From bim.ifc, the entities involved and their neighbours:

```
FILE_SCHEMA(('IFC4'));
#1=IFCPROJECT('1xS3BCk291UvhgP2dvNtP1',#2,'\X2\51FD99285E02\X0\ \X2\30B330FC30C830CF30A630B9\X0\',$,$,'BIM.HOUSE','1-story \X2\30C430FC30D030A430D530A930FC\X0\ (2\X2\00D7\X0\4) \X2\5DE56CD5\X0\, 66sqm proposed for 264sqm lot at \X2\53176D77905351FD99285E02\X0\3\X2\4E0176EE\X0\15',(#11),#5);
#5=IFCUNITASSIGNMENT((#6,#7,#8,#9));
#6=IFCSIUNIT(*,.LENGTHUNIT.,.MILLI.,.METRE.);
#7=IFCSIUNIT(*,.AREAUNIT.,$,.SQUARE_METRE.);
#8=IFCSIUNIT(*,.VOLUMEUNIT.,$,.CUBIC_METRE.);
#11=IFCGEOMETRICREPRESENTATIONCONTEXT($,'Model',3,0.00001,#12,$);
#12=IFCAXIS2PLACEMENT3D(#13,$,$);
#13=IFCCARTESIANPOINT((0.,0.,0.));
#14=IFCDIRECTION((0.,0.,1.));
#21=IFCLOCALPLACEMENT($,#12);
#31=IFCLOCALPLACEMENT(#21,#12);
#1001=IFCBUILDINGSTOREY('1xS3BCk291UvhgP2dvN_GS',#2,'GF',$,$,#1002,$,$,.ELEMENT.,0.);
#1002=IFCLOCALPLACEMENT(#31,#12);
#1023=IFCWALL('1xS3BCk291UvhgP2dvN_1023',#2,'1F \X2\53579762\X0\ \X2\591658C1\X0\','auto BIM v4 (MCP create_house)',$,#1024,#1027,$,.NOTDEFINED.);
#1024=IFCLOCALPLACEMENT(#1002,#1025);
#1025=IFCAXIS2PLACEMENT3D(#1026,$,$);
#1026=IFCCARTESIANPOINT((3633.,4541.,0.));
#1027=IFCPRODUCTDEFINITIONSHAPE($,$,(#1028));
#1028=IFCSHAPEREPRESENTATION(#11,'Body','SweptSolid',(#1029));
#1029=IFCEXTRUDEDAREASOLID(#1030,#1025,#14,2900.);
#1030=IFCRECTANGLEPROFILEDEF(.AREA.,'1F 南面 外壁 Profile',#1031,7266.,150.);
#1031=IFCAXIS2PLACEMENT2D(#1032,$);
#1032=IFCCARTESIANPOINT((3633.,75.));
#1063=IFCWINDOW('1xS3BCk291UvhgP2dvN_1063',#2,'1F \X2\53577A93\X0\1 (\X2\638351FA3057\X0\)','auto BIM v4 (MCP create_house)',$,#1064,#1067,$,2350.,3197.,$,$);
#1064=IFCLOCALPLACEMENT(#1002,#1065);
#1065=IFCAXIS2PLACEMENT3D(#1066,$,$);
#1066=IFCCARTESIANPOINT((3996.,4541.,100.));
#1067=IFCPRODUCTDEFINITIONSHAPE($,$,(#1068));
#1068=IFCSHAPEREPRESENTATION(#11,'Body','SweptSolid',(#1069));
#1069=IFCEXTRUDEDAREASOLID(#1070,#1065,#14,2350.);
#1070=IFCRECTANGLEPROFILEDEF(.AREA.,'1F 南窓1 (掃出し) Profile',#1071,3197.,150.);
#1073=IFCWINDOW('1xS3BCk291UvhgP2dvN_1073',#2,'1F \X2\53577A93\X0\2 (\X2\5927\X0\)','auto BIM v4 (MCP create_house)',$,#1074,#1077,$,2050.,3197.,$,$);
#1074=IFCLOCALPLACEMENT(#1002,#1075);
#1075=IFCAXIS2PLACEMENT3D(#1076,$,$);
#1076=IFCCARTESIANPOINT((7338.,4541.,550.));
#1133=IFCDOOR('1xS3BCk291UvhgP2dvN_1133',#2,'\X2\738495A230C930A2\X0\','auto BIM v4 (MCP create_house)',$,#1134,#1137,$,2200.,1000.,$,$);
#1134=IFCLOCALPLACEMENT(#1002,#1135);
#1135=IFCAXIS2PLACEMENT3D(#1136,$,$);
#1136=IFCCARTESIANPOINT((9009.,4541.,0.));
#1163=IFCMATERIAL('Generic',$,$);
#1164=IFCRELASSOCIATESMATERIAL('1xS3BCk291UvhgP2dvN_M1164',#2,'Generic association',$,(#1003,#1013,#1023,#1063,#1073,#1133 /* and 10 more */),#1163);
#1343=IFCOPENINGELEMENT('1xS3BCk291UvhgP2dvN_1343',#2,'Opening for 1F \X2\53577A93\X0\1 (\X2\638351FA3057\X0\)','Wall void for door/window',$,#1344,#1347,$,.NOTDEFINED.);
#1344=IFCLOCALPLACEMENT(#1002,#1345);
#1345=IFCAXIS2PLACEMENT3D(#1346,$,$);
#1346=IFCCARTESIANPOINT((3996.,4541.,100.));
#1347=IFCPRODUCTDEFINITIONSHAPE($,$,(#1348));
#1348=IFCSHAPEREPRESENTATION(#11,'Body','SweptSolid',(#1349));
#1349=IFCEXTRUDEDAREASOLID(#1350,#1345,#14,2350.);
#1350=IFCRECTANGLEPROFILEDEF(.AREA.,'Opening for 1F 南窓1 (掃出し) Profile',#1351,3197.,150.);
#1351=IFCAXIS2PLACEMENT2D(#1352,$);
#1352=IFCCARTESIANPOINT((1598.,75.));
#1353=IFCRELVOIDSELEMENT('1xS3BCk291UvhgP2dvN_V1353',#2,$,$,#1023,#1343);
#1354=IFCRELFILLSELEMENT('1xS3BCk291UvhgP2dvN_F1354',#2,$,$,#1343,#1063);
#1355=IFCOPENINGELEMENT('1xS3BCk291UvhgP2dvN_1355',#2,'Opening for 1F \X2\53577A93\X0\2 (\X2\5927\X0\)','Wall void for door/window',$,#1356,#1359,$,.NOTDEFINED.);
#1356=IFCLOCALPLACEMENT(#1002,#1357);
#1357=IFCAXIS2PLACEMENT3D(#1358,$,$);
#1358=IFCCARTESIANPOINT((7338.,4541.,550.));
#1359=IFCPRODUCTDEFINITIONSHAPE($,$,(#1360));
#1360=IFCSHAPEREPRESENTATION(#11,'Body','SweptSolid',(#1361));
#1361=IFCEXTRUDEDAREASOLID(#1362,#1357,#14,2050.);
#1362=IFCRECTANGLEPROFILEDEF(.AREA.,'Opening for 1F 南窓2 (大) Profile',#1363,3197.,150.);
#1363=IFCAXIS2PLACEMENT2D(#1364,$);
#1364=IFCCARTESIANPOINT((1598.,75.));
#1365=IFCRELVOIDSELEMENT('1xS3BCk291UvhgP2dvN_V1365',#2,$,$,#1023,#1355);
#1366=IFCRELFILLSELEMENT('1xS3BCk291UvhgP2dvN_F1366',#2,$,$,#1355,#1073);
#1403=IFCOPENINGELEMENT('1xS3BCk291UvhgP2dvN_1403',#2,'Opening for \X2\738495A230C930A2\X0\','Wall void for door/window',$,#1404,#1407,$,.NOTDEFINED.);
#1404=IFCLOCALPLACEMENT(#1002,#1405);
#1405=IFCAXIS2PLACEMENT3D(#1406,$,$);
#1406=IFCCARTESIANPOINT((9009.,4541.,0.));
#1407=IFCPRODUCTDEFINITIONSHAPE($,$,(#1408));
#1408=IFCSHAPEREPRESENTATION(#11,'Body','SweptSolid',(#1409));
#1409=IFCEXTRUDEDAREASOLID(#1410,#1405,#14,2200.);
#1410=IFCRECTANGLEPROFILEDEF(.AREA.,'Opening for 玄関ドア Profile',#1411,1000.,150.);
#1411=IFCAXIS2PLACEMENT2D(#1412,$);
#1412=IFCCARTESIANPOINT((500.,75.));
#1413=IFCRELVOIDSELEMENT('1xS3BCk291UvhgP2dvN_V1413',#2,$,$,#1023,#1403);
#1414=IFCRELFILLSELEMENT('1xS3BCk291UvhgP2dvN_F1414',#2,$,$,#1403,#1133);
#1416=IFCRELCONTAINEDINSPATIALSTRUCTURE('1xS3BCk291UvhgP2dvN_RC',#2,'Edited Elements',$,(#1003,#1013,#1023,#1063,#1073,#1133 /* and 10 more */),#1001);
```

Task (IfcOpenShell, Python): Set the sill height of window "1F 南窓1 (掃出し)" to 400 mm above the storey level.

```python
import numpy as np
import ifcopenshell
import ifcopenshell.api.geometry
import ifcopenshell.geom
import ifcopenshell.util.element
import ifcopenshell.util.placement
import ifcopenshell.util.shape
import ifcopenshell.util.unit

model = ifcopenshell.open("bim.ifc")
unit_scale = ifcopenshell.util.unit.calculate_unit_scale(model)

window = model.by_guid("1xS3BCk291UvhgP2dvN_1063")
opening = window.FillsVoids[0].RelatingOpeningElement
storey = ifcopenshell.util.element.get_container(window, ifc_class="IfcBuildingStorey")
level = ifcopenshell.util.placement.get_local_placement(storey.ObjectPlacement)[2, 3]

# The opening's origin need not be at the sill, so measure its lowest point.
shape = ifcopenshell.geom.create_shape(ifcopenshell.geom.settings(), opening)
bottom = ifcopenshell.util.shape.get_shape_bottom_elevation(shape, shape.geometry) / unit_scale
dz = level + 0.4 / unit_scale - bottom

shift = np.array([0.0, 0.0, dz])
# The window is not placed relative to its opening, so move both.
for product in (opening, window):
    matrix = ifcopenshell.util.placement.get_local_placement(product.ObjectPlacement)
    matrix[:3, 3] += shift
    ifcopenshell.api.geometry.edit_object_placement(model, product=product, matrix=matrix, is_si=False)

print(f"moved by {dz * unit_scale:+.3f} m")

model.write("bim_rev.ifc")
```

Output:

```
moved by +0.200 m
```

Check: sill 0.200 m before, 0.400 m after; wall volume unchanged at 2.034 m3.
